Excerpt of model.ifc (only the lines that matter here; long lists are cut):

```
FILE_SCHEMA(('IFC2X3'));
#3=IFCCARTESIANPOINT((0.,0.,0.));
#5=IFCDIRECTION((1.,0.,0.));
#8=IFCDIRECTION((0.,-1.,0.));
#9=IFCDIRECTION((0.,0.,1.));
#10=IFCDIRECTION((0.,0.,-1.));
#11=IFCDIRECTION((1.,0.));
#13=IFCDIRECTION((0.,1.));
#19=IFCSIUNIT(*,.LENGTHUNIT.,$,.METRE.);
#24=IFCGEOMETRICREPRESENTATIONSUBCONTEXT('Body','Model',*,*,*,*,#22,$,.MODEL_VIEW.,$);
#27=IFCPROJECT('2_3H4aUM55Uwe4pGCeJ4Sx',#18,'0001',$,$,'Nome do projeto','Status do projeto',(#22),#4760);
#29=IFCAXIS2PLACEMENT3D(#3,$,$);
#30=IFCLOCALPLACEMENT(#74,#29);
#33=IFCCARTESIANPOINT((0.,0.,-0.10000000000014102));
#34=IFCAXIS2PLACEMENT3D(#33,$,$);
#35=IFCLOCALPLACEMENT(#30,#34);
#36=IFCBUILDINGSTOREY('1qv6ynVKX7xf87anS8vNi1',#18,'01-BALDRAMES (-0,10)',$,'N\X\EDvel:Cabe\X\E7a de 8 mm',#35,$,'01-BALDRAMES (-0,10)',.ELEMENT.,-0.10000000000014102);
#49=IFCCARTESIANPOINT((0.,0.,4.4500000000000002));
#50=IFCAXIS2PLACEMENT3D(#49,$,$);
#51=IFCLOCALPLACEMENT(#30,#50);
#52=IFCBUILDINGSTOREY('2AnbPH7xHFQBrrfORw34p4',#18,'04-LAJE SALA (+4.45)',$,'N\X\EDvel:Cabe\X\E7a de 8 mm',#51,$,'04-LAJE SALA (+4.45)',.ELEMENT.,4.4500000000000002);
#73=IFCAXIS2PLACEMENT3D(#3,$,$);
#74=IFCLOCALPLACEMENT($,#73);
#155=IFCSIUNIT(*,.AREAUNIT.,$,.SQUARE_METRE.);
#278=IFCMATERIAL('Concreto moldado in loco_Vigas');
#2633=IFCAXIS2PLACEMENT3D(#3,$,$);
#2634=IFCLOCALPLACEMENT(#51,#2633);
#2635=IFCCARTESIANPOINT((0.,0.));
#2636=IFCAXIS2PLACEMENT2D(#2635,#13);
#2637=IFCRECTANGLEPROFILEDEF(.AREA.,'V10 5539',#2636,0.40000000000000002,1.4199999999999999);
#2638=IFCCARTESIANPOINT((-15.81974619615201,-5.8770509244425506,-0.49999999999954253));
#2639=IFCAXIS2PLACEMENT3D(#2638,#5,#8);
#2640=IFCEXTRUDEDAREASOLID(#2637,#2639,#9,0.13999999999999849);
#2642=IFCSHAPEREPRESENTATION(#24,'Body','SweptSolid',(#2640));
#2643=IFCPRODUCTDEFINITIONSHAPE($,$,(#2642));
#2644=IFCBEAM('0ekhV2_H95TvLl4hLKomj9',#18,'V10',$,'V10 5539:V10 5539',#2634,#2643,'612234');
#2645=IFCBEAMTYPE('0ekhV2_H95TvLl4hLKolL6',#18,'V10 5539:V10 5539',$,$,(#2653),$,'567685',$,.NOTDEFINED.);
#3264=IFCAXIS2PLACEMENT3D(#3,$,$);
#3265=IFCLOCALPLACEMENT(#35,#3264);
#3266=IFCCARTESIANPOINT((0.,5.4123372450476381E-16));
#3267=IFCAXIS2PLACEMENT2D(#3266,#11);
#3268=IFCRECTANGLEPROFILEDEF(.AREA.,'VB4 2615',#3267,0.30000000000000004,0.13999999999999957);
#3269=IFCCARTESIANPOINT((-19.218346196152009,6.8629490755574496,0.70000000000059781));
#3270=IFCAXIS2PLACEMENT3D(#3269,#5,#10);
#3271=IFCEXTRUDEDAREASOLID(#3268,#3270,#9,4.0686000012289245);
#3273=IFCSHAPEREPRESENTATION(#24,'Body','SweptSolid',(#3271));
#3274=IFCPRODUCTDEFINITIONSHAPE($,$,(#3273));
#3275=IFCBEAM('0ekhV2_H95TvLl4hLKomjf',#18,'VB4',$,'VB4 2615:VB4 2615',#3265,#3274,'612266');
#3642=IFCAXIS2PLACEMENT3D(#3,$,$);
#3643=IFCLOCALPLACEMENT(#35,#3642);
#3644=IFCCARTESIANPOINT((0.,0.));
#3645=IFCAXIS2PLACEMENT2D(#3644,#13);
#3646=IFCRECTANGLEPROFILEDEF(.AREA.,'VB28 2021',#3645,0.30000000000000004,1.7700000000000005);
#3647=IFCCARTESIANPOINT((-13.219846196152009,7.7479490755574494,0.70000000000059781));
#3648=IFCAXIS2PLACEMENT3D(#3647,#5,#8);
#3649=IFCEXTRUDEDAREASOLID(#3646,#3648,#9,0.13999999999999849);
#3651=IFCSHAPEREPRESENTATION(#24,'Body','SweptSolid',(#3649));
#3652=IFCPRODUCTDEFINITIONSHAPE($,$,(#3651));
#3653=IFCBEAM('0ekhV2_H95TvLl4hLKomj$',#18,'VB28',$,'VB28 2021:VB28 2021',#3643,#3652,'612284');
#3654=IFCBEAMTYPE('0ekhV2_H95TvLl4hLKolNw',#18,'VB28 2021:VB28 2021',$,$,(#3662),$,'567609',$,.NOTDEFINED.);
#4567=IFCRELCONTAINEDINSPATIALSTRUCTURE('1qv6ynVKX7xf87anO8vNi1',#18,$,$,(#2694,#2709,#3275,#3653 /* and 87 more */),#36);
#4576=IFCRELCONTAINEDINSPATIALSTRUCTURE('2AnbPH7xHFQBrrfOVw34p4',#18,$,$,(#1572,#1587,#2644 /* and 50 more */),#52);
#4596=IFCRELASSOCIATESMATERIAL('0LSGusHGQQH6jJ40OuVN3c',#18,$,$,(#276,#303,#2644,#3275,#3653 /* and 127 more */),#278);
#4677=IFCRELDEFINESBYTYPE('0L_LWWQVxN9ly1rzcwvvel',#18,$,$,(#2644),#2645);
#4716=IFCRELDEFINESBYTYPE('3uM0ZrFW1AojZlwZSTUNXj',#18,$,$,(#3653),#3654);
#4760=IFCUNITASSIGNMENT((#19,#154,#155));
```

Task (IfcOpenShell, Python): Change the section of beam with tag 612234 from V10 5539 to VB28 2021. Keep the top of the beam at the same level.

```python
import ifcopenshell
import ifcopenshell.api.type
import ifcopenshell.util.element
import ifcopenshell.util.representation

model = ifcopenshell.open("model.ifc")

member = model.by_guid("0ekhV2_H95TvLl4hLKomj9")
source = next(p for p in model.by_type("IfcRectangleProfileDef") if p.ProfileName == "VB28 2021")

body = ifcopenshell.util.representation.get_representation(member, "Model", "Body")
solid = body.Items[0]
old_profile = solid.SweptArea

# Copy the section's sizes but keep this member's own profile position.
profile = ifcopenshell.util.element.copy(model, source)
# Profiles are centred, so shift by half the change in depth to hold the top.
shift = (old_profile.XDim - profile.XDim) / 2
x, y = old_profile.Position.Location.Coordinates
up = (0.0, -1.0)  # upwards, in the solid's own plane
location = model.createIfcCartesianPoint((x + up[0] * shift, y + up[1] * shift))
profile.Position = model.createIfcAxis2Placement2D(location, old_profile.Position.RefDirection)
solid.SweptArea = profile
if not model.get_total_inverses(old_profile):
    ifcopenshell.util.element.remove_deep2(model, old_profile)

new_type = model.by_guid("0ekhV2_H95TvLl4hLKolNw")
ifcopenshell.api.type.assign_type(
    model, related_objects=[member], relating_type=new_type, should_map_representations=False
)
member.ObjectType = "VB28 2021:VB28 2021"

print(solid.SweptArea)

model.write("model-out.ifc")
```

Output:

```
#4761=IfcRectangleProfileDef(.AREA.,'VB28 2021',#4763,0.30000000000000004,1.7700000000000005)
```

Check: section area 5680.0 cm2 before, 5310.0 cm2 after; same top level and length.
